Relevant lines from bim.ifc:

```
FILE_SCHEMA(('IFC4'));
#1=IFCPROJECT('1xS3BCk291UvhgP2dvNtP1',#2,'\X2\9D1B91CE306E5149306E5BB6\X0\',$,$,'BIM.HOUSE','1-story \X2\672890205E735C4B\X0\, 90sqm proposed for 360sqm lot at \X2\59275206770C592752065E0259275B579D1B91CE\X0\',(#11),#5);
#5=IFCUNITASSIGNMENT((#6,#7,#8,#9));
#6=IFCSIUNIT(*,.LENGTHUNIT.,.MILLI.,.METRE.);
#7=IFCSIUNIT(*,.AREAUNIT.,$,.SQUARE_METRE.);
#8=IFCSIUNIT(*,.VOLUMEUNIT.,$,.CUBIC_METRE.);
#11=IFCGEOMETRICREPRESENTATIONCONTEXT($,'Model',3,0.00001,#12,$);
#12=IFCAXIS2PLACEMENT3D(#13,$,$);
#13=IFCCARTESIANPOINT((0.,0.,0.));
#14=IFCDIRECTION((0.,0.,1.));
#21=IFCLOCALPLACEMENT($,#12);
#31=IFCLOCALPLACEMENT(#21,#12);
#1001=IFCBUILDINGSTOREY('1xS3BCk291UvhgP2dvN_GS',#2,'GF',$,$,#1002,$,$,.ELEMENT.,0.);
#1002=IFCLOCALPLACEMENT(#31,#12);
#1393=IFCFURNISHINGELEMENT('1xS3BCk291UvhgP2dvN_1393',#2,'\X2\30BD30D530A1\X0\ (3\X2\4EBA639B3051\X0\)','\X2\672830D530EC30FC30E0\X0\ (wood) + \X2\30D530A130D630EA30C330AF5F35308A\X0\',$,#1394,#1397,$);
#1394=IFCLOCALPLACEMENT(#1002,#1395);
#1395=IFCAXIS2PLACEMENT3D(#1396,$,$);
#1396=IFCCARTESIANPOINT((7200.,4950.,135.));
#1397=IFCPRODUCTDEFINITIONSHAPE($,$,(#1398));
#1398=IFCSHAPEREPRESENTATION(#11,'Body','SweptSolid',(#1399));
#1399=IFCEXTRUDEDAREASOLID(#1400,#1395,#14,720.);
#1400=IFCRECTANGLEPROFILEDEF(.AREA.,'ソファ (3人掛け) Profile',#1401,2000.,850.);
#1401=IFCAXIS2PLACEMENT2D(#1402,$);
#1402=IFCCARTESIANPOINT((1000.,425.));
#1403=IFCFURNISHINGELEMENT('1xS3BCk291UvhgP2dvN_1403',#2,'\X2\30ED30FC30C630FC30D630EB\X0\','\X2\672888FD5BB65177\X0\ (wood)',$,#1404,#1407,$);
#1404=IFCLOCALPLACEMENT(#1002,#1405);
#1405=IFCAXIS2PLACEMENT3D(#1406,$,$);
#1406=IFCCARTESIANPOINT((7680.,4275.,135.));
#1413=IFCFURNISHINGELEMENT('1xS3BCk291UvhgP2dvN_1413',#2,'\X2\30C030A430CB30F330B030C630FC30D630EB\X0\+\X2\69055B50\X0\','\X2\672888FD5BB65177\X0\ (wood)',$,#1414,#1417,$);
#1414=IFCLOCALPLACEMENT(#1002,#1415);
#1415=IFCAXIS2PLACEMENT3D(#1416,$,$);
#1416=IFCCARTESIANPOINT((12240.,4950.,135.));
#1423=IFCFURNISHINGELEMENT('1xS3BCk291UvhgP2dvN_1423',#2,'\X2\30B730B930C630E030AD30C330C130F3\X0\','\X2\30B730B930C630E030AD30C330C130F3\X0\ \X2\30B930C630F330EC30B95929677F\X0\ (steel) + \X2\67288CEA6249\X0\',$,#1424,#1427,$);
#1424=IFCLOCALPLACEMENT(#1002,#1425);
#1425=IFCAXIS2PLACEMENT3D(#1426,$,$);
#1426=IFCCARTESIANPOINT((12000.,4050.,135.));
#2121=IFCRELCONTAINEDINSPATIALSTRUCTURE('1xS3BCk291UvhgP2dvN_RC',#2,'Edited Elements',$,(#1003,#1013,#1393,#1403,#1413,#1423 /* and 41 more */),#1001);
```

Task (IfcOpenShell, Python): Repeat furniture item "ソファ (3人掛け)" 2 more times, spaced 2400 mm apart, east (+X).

```python
import numpy as np
import ifcopenshell
import ifcopenshell.api.geometry
import ifcopenshell.api.root
import ifcopenshell.util.element
import ifcopenshell.util.placement

model = ifcopenshell.open("bim.ifc")


def reuse_history(source, copy):
    """copy_class also copies each property set's owner history, people and application; keep the originals."""
    for rel in copy.IsDefinedBy:
        if rel.is_a("IfcRelDefinesByProperties") and (history := rel.RelatingPropertyDefinition.OwnerHistory):
            rel.RelatingPropertyDefinition.OwnerHistory = source.OwnerHistory
            ifcopenshell.util.element.remove_deep2(model, history)


source = model.by_guid("1xS3BCk291UvhgP2dvN_1393")
base = ifcopenshell.util.placement.get_local_placement(source.ObjectPlacement)
step = np.array([1.0, 0.0, 0.0]) * 2400.0

for i in range(1, 3):
    copy = ifcopenshell.api.root.copy_class(model, product=source)
    copy.Representation = ifcopenshell.util.element.copy_deep(
        model, source.Representation, exclude=["IfcGeometricRepresentationContext", "IfcRepresentationMap"]
    )
    reuse_history(source, copy)
    matrix = base.copy()
    matrix[:3, 3] += i * step
    print("added at", matrix[:3, 3].round(3) + 0.0)
    ifcopenshell.api.geometry.edit_object_placement(model, product=copy, matrix=matrix, is_si=False)

model.write("bim_edited.ifc")
```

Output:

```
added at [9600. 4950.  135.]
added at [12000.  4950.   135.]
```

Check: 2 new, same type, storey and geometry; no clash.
